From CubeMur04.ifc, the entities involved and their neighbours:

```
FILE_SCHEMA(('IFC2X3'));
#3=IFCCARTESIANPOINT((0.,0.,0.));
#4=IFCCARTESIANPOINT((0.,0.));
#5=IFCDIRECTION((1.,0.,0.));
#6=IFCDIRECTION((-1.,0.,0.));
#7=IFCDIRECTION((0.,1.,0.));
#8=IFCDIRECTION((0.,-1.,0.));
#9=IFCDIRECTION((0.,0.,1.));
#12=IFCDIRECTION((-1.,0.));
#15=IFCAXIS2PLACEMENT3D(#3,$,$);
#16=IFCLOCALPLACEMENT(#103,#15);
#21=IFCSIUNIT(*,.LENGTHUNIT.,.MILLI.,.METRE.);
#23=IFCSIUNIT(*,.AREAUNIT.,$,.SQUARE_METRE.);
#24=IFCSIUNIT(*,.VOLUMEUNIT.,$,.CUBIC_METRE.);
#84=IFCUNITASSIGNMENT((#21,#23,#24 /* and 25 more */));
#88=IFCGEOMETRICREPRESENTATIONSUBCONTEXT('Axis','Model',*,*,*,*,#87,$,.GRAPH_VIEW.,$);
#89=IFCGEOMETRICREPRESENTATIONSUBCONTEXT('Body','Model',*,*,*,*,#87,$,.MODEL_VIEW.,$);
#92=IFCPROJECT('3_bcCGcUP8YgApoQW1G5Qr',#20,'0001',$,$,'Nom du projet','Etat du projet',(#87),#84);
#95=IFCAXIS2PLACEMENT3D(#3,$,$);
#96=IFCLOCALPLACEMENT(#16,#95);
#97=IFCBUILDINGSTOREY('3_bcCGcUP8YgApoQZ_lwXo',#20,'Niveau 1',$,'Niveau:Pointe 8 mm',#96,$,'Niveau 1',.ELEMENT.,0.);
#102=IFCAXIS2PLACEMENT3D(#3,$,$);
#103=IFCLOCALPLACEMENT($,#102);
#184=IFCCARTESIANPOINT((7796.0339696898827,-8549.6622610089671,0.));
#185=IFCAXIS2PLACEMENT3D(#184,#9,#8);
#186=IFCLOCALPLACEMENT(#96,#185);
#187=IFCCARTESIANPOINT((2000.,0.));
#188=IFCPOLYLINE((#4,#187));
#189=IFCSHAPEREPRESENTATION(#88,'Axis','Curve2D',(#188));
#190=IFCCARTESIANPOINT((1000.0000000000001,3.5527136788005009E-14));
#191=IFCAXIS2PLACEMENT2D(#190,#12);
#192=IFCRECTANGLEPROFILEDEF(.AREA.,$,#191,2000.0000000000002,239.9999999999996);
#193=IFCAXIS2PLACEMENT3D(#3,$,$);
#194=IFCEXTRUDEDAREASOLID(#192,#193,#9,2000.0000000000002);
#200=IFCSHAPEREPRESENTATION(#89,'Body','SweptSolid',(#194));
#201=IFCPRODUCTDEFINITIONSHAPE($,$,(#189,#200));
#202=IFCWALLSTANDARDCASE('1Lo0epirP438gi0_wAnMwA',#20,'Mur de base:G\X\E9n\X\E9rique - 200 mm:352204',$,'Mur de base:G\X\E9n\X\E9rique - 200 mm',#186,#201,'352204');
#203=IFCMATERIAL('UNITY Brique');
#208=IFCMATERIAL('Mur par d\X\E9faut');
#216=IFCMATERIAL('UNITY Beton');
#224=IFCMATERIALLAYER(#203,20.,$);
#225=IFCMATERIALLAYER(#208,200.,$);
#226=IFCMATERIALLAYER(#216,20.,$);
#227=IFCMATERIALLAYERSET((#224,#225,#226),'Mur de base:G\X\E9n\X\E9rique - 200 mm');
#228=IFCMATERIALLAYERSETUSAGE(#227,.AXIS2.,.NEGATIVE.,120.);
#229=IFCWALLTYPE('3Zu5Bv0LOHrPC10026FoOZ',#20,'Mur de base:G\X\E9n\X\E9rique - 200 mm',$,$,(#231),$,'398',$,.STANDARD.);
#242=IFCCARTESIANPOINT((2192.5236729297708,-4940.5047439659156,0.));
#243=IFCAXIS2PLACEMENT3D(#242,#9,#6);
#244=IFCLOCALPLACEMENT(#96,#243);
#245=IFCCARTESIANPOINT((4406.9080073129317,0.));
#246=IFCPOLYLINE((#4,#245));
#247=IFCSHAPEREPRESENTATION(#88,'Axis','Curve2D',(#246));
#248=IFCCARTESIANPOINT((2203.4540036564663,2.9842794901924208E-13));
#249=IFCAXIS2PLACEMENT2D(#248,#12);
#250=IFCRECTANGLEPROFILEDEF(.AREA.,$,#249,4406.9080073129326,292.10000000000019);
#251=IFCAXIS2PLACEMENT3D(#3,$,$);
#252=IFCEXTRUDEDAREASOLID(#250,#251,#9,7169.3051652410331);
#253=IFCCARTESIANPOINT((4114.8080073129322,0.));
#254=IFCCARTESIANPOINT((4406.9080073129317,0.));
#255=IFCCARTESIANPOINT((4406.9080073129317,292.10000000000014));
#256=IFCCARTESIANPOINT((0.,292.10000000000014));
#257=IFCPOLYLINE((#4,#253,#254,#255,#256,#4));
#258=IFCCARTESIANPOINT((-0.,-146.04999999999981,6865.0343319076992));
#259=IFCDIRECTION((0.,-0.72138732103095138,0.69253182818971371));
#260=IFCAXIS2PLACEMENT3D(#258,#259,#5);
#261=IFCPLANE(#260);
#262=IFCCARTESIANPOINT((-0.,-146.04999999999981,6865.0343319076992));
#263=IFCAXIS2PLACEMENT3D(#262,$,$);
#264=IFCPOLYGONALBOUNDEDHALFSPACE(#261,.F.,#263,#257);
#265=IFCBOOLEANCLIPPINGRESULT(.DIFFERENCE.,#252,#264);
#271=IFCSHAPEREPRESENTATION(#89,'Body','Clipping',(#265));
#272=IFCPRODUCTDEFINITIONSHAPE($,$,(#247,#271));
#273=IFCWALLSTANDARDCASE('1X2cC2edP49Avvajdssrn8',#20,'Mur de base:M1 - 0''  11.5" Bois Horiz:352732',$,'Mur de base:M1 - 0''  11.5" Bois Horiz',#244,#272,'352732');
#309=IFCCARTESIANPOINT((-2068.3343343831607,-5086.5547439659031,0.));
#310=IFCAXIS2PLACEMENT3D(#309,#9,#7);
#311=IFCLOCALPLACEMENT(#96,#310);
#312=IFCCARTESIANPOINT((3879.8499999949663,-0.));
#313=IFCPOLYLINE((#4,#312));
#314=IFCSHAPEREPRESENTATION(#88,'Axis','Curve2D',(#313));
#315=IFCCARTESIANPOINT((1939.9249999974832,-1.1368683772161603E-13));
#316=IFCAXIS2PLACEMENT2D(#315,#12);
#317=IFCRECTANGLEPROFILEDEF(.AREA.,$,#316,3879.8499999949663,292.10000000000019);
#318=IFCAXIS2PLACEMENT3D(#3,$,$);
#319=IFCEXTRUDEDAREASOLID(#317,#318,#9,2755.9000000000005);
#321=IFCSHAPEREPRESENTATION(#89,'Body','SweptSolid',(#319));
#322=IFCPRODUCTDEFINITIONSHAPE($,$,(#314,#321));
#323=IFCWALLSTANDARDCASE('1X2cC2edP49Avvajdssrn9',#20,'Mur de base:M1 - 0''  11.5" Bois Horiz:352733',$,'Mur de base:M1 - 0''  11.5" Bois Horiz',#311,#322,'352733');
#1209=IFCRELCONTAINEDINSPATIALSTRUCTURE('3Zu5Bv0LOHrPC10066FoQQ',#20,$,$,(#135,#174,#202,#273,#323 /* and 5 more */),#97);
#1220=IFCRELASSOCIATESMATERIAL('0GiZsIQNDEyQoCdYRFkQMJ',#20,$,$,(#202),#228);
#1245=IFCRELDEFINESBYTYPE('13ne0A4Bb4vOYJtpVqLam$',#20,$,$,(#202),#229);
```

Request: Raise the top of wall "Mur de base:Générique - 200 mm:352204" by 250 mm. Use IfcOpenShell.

```python
import ifcopenshell
import ifcopenshell.geom
import ifcopenshell.util.representation
import ifcopenshell.util.shape
import ifcopenshell.util.unit

model = ifcopenshell.open("CubeMur04.ifc")
unit_scale = ifcopenshell.util.unit.calculate_unit_scale(model)
settings = ifcopenshell.geom.settings()


def volume(element):
    """Net volume in cubic metres, openings subtracted."""
    shape = ifcopenshell.geom.create_shape(settings, element)
    return ifcopenshell.util.shape.get_volume(shape.geometry)


wall = model.by_id(202)
before = volume(wall)

body = ifcopenshell.util.representation.get_representation(wall, "Model", "Body")
solid = body.Items[0]
old_height = solid.Depth
solid.Depth += 0.25 / unit_scale
after = volume(wall)

print(f"height {old_height:g} -> {solid.Depth:g}, volume {before:.3f} -> {after:.3f} m3")

model.write("CubeMur04_rev.ifc")
```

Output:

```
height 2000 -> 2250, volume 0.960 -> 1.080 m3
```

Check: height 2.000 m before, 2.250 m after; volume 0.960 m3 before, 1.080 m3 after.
